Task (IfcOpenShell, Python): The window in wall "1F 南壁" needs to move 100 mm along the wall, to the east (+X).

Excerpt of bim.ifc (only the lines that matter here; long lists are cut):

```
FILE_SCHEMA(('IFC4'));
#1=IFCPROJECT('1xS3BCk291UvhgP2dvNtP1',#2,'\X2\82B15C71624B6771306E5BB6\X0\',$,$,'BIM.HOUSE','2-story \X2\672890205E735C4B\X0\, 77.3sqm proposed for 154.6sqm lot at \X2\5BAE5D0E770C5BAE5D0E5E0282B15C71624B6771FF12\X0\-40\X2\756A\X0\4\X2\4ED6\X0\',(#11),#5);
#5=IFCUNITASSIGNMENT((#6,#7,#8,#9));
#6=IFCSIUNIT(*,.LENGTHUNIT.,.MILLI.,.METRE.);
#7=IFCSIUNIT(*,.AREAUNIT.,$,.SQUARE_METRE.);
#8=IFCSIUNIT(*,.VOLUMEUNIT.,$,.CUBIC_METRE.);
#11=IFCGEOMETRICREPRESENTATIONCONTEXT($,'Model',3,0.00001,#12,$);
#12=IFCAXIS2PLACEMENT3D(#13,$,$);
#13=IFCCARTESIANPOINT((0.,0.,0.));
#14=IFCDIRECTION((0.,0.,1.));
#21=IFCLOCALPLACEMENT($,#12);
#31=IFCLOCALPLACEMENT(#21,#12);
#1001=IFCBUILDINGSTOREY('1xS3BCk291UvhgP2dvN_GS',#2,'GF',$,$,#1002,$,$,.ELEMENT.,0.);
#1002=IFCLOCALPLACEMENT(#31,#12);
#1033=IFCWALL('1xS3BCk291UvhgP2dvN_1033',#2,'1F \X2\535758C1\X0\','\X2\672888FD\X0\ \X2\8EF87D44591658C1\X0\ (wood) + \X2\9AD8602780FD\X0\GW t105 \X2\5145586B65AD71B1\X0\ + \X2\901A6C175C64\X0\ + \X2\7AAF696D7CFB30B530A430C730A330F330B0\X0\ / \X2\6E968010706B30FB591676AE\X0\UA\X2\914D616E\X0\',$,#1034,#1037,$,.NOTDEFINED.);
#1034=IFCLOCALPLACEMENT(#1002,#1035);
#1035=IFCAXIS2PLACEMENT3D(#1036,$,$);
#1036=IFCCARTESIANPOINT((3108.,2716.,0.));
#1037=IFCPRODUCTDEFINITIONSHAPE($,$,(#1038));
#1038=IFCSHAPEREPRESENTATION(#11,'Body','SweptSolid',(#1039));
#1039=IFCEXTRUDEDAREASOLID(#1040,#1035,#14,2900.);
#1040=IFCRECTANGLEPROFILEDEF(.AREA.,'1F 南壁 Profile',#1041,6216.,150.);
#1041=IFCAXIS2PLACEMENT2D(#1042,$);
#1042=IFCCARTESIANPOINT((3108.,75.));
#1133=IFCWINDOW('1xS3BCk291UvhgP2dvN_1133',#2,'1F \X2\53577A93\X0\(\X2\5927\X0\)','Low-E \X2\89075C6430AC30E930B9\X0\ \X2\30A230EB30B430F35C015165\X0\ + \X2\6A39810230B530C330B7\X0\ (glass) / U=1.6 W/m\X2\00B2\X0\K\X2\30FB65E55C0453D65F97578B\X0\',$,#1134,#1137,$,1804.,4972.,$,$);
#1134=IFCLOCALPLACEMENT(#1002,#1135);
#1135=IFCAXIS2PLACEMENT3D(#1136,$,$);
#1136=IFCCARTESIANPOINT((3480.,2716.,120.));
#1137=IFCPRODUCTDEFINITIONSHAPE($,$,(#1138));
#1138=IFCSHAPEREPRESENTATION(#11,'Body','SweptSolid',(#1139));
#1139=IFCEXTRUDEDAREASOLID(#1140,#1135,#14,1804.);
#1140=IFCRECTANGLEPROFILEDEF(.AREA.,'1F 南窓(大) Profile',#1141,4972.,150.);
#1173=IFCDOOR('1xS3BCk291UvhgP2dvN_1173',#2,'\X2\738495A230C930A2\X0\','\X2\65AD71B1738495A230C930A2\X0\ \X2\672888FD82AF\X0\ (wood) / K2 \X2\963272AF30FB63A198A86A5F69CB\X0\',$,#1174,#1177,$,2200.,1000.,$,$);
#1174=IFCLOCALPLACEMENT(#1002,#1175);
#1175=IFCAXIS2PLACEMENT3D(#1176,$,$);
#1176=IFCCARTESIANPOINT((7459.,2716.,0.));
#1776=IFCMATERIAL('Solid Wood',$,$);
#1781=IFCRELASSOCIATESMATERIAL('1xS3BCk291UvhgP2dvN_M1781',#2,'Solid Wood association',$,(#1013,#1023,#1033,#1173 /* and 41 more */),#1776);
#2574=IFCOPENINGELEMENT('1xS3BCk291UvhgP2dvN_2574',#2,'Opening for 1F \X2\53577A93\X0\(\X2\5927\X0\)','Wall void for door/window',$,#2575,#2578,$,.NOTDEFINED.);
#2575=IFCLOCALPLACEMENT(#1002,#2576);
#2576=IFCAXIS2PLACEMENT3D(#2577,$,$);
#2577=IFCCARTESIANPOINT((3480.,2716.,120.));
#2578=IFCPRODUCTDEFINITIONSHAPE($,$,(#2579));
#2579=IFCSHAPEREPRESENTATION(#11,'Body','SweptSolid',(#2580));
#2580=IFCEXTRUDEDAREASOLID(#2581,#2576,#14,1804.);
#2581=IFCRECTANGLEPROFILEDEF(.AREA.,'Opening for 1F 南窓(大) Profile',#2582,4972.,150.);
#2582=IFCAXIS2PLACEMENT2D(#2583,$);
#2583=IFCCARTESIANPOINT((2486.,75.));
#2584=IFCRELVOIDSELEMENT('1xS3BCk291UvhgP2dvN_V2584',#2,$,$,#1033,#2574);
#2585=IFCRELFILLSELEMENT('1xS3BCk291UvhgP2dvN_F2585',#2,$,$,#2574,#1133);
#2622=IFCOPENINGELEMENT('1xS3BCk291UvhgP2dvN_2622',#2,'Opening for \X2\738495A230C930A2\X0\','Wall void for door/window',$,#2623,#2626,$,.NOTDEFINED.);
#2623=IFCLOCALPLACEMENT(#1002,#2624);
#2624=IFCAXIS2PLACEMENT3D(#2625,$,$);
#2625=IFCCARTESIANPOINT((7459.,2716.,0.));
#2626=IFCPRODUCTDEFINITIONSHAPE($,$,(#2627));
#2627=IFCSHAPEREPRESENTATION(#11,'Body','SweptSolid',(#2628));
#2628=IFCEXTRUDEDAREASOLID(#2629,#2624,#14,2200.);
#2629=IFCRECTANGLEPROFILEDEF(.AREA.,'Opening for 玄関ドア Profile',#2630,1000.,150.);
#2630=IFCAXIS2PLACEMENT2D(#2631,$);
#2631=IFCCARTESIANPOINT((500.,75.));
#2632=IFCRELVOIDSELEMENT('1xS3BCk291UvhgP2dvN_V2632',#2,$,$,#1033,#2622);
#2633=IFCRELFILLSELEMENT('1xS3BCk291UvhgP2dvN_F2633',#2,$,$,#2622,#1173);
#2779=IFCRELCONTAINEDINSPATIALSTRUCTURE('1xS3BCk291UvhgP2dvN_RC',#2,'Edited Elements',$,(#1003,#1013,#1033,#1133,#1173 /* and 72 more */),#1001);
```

```python
import ifcopenshell
import ifcopenshell.api.geometry
import ifcopenshell.util.placement

model = ifcopenshell.open("bim.ifc")

window = model.by_guid("1xS3BCk291UvhgP2dvN_1133")
opening = window.FillsVoids[0].RelatingOpeningElement
wall = opening.VoidsElements[0].RelatingBuildingElement

wall_matrix = ifcopenshell.util.placement.get_local_placement(wall.ObjectPlacement)
shift = wall_matrix[:3, 0] * 100.0
before = ifcopenshell.util.placement.get_local_placement(window.ObjectPlacement)[:3, 3].copy()

# The window is not placed relative to its opening, so move both.
for product in (opening, window):
    matrix = ifcopenshell.util.placement.get_local_placement(product.ObjectPlacement)
    matrix[:3, 3] += shift
    ifcopenshell.api.geometry.edit_object_placement(model, product=product, matrix=matrix, is_si=False)

after = ifcopenshell.util.placement.get_local_placement(window.ObjectPlacement)[:3, 3]
print("window moved by", (after - before).round(3) + 0.0)

model.write("bim_edited.ifc")
```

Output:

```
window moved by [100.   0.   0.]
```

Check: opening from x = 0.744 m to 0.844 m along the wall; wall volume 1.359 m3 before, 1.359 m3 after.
